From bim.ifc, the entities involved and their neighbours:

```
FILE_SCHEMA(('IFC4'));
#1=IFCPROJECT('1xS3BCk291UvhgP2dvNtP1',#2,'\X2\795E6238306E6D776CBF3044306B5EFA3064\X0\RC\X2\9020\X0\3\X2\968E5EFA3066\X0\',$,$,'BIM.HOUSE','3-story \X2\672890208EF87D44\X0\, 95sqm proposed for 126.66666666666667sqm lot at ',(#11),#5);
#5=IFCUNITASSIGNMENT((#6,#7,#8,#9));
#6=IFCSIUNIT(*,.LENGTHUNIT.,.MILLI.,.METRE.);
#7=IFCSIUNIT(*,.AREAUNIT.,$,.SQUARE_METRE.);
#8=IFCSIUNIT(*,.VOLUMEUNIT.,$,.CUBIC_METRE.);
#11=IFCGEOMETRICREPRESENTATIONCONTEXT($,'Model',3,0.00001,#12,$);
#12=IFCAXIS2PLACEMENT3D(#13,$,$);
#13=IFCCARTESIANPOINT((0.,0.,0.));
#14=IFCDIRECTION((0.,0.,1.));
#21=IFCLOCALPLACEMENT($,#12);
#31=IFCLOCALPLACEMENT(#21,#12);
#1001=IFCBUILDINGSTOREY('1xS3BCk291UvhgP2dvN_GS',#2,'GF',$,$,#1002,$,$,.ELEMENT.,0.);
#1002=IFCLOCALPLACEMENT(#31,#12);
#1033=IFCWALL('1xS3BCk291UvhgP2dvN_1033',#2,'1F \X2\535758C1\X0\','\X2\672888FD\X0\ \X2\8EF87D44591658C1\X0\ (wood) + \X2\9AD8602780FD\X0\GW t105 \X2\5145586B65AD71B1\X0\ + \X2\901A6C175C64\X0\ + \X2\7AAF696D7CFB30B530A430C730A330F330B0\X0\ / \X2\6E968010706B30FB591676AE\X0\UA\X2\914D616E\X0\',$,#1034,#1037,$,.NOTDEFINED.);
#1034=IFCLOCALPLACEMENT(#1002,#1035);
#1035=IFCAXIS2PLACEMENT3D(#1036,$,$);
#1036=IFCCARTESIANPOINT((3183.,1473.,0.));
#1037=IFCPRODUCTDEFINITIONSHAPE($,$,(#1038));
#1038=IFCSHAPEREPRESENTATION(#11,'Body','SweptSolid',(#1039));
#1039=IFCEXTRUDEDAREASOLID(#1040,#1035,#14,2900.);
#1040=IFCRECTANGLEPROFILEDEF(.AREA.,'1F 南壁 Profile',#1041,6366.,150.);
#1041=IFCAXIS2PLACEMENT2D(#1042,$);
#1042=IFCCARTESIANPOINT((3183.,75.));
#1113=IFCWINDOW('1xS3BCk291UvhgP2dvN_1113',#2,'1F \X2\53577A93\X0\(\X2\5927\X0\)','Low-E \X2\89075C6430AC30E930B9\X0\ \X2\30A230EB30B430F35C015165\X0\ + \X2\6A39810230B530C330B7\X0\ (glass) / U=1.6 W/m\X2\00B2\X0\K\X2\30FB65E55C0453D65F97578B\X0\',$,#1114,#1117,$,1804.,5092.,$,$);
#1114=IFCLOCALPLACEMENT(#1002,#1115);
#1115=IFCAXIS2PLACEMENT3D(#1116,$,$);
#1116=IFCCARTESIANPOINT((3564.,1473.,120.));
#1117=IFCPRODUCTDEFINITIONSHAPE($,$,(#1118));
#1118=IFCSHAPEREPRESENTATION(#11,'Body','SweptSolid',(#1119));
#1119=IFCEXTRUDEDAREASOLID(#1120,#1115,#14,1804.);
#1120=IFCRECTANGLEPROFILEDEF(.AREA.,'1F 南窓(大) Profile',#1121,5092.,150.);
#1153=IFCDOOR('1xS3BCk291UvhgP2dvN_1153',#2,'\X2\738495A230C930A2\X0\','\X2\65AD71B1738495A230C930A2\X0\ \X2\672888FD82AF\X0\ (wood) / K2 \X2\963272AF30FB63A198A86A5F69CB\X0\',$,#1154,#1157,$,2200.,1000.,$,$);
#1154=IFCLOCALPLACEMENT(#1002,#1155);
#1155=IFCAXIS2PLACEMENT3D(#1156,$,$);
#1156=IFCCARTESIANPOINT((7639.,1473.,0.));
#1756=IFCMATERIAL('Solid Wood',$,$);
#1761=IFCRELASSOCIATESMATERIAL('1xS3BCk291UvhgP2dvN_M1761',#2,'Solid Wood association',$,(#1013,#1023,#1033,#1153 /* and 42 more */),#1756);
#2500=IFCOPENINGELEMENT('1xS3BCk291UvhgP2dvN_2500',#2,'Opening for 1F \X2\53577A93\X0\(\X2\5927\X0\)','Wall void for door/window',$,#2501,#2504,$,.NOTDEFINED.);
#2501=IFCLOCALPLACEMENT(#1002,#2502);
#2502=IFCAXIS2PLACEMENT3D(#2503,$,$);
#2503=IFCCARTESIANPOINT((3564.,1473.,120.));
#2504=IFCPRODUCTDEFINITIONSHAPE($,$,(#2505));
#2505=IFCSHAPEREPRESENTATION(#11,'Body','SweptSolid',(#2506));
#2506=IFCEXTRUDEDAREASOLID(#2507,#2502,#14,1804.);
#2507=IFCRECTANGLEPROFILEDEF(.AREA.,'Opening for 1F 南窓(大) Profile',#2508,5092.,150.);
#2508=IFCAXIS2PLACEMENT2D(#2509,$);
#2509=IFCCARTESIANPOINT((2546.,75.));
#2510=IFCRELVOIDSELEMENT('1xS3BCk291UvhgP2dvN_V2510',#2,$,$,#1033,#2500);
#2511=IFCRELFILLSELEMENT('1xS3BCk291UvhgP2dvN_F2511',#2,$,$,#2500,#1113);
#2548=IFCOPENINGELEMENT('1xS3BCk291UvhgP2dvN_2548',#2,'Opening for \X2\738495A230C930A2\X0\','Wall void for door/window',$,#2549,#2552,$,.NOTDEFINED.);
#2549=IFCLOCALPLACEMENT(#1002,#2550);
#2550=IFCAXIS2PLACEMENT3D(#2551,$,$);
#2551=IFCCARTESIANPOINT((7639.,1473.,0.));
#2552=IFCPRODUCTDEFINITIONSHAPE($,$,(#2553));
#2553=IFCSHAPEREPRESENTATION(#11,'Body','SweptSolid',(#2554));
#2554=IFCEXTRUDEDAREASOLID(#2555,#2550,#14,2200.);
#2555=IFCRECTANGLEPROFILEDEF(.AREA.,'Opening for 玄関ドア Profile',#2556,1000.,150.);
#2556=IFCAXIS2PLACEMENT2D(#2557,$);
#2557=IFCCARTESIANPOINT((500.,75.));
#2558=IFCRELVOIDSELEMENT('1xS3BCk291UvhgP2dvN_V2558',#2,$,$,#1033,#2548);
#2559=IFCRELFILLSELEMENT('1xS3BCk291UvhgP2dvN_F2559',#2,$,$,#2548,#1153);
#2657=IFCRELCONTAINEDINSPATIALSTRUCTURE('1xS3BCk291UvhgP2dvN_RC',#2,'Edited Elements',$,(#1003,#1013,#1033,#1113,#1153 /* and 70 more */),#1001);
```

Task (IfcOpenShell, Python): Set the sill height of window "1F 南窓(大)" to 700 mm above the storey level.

```python
import numpy as np
import ifcopenshell
import ifcopenshell.api.geometry
import ifcopenshell.geom
import ifcopenshell.util.element
import ifcopenshell.util.placement
import ifcopenshell.util.shape
import ifcopenshell.util.unit

model = ifcopenshell.open("bim.ifc")
unit_scale = ifcopenshell.util.unit.calculate_unit_scale(model)

window = model.by_guid("1xS3BCk291UvhgP2dvN_1113")
opening = window.FillsVoids[0].RelatingOpeningElement
storey = ifcopenshell.util.element.get_container(window, ifc_class="IfcBuildingStorey")
level = ifcopenshell.util.placement.get_local_placement(storey.ObjectPlacement)[2, 3]

# The opening's origin need not be at the sill, so measure its lowest point.
shape = ifcopenshell.geom.create_shape(ifcopenshell.geom.settings(), opening)
bottom = ifcopenshell.util.shape.get_shape_bottom_elevation(shape, shape.geometry) / unit_scale
dz = level + 0.7 / unit_scale - bottom

shift = np.array([0.0, 0.0, dz])
# The window is not placed relative to its opening, so move both.
for product in (opening, window):
    matrix = ifcopenshell.util.placement.get_local_placement(product.ObjectPlacement)
    matrix[:3, 3] += shift
    ifcopenshell.api.geometry.edit_object_placement(model, product=product, matrix=matrix, is_si=False)

print(f"moved by {dz * unit_scale:+.3f} m")

model.write("bim_edited.ifc")
```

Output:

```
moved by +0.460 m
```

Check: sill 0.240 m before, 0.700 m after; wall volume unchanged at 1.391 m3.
